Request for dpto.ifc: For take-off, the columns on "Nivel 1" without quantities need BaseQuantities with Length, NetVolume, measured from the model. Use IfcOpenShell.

First a look at what the model holds.

```python
import ifcopenshell
import ifcopenshell.util.element
import ifcopenshell.util.unit

model = ifcopenshell.open("dpto.ifc")
print(model.schema)
for unit_type in ("LENGTHUNIT", "AREAUNIT", "VOLUMEUNIT"):
    print(unit_type, ifcopenshell.util.unit.calculate_unit_scale(model, unit_type))
storey = next(s for s in model.by_type("IfcBuildingStorey") if s.Name == "Nivel 1")
columns = [e for e in ifcopenshell.util.element.get_decomposition(storey) if e.is_a("IfcColumn")]
for e in sorted(columns, key=lambda e: e.id()):
    print(e.id(), e.is_a(), e.Name, list(ifcopenshell.util.element.get_psets(e, qtos_only=True)), sep=" | ")
```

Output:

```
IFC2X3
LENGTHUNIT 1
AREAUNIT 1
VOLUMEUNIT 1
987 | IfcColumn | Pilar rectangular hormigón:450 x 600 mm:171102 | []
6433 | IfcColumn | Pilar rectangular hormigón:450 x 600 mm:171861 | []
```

```python
import ifcopenshell
import ifcopenshell.api.pset
import ifcopenshell.geom
import ifcopenshell.util.element
import ifcopenshell.util.shape
import ifcopenshell.util.unit

model = ifcopenshell.open("dpto.ifc")
unit_scale = ifcopenshell.util.unit.calculate_unit_scale(model)
volume_scale = ifcopenshell.util.unit.calculate_unit_scale(model, "VOLUMEUNIT")
settings = ifcopenshell.geom.settings()

storey = next(s for s in model.by_type("IfcBuildingStorey") if s.Name == "Nivel 1")
columns = [e for e in ifcopenshell.util.element.get_decomposition(storey) if e.is_a("IfcColumn")]

for e in sorted(columns, key=lambda e: e.id()):
    if ifcopenshell.util.element.get_psets(e, qtos_only=True, should_inherit=False):
        continue
    # Geometry comes back in metres, in the element's own axes.
    shape = ifcopenshell.geom.create_shape(settings, e)
    values = {
        "Length": ifcopenshell.util.shape.get_z(shape.geometry) / unit_scale,
        "NetVolume": ifcopenshell.util.shape.get_volume(shape.geometry) / volume_scale,
    }
    qto = ifcopenshell.api.pset.add_qto(model, product=e, name="BaseQuantities")
    ifcopenshell.api.pset.edit_qto(model, qto=qto, properties=values)
    print(e.id(), {k: round(v, 3) for k, v in values.items()})

model.write("dpto_v2.ifc")
```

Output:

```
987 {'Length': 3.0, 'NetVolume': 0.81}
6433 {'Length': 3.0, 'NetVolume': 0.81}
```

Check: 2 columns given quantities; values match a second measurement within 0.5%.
